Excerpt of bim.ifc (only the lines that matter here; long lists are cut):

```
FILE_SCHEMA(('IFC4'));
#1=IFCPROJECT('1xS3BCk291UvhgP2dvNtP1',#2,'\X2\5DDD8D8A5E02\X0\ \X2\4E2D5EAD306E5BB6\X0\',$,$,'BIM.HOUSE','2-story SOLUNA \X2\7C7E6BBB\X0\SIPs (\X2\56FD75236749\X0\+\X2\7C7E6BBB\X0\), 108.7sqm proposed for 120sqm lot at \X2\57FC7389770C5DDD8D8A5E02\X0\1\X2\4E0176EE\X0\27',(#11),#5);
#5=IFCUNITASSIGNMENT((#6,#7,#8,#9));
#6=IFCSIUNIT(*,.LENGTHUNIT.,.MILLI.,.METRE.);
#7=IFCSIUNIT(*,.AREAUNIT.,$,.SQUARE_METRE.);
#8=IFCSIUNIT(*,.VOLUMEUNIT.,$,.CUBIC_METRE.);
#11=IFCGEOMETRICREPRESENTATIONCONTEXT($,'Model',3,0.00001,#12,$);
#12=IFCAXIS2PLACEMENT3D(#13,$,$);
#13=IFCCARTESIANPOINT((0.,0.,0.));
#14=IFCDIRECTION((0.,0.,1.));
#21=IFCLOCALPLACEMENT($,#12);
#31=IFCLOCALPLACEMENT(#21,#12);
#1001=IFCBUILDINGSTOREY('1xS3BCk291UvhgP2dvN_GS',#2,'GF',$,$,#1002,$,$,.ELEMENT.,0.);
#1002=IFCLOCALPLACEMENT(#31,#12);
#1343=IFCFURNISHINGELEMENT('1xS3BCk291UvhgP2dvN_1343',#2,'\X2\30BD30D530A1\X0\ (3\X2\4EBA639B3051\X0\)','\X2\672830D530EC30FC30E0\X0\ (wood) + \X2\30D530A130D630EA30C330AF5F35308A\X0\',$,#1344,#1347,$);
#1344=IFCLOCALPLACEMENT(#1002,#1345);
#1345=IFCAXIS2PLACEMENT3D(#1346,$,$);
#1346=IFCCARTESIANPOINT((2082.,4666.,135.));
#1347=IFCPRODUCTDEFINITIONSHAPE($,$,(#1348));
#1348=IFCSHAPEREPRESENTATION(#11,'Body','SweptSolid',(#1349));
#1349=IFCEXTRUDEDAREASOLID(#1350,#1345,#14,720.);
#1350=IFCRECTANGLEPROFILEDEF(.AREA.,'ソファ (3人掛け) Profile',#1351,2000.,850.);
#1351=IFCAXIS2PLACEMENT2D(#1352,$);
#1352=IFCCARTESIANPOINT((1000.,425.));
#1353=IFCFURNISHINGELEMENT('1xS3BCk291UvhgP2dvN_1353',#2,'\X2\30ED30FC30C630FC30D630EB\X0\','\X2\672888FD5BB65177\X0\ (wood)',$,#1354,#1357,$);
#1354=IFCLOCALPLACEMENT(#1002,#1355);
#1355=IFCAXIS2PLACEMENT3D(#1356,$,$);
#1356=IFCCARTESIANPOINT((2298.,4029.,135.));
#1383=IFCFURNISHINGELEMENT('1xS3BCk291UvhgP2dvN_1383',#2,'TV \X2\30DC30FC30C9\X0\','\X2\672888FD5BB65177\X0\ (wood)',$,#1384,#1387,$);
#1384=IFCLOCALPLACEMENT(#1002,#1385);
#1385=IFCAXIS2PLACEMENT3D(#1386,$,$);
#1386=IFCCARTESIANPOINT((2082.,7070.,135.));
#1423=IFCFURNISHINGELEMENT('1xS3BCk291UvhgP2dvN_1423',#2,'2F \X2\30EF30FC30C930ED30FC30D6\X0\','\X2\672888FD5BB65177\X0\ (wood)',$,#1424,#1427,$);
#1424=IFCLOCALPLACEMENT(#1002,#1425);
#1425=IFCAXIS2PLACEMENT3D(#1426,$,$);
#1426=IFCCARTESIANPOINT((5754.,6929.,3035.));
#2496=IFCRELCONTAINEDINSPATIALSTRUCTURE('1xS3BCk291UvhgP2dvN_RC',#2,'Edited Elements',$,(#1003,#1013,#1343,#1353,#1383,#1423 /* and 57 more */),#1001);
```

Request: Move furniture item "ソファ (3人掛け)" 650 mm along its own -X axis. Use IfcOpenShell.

```python
import ifcopenshell
import ifcopenshell.api.geometry
import ifcopenshell.util.placement
import ifcopenshell.util.unit

model = ifcopenshell.open("bim.ifc")
unit_scale = ifcopenshell.util.unit.calculate_unit_scale(model)

item = model.by_id(1343)
matrix = ifcopenshell.util.placement.get_local_placement(item.ObjectPlacement)
matrix[:3, 3] -= matrix[:3, 0] * 0.65 / unit_scale
ifcopenshell.api.geometry.edit_object_placement(model, product=item, matrix=matrix, is_si=False)

print(ifcopenshell.util.placement.get_local_placement(item.ObjectPlacement).round(3) + 0.0)

model.write("bim_updated.ifc")
```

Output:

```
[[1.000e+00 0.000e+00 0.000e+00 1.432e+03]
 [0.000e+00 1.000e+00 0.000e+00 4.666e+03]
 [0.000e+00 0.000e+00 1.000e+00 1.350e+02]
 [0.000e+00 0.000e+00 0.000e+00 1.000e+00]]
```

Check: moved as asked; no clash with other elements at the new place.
